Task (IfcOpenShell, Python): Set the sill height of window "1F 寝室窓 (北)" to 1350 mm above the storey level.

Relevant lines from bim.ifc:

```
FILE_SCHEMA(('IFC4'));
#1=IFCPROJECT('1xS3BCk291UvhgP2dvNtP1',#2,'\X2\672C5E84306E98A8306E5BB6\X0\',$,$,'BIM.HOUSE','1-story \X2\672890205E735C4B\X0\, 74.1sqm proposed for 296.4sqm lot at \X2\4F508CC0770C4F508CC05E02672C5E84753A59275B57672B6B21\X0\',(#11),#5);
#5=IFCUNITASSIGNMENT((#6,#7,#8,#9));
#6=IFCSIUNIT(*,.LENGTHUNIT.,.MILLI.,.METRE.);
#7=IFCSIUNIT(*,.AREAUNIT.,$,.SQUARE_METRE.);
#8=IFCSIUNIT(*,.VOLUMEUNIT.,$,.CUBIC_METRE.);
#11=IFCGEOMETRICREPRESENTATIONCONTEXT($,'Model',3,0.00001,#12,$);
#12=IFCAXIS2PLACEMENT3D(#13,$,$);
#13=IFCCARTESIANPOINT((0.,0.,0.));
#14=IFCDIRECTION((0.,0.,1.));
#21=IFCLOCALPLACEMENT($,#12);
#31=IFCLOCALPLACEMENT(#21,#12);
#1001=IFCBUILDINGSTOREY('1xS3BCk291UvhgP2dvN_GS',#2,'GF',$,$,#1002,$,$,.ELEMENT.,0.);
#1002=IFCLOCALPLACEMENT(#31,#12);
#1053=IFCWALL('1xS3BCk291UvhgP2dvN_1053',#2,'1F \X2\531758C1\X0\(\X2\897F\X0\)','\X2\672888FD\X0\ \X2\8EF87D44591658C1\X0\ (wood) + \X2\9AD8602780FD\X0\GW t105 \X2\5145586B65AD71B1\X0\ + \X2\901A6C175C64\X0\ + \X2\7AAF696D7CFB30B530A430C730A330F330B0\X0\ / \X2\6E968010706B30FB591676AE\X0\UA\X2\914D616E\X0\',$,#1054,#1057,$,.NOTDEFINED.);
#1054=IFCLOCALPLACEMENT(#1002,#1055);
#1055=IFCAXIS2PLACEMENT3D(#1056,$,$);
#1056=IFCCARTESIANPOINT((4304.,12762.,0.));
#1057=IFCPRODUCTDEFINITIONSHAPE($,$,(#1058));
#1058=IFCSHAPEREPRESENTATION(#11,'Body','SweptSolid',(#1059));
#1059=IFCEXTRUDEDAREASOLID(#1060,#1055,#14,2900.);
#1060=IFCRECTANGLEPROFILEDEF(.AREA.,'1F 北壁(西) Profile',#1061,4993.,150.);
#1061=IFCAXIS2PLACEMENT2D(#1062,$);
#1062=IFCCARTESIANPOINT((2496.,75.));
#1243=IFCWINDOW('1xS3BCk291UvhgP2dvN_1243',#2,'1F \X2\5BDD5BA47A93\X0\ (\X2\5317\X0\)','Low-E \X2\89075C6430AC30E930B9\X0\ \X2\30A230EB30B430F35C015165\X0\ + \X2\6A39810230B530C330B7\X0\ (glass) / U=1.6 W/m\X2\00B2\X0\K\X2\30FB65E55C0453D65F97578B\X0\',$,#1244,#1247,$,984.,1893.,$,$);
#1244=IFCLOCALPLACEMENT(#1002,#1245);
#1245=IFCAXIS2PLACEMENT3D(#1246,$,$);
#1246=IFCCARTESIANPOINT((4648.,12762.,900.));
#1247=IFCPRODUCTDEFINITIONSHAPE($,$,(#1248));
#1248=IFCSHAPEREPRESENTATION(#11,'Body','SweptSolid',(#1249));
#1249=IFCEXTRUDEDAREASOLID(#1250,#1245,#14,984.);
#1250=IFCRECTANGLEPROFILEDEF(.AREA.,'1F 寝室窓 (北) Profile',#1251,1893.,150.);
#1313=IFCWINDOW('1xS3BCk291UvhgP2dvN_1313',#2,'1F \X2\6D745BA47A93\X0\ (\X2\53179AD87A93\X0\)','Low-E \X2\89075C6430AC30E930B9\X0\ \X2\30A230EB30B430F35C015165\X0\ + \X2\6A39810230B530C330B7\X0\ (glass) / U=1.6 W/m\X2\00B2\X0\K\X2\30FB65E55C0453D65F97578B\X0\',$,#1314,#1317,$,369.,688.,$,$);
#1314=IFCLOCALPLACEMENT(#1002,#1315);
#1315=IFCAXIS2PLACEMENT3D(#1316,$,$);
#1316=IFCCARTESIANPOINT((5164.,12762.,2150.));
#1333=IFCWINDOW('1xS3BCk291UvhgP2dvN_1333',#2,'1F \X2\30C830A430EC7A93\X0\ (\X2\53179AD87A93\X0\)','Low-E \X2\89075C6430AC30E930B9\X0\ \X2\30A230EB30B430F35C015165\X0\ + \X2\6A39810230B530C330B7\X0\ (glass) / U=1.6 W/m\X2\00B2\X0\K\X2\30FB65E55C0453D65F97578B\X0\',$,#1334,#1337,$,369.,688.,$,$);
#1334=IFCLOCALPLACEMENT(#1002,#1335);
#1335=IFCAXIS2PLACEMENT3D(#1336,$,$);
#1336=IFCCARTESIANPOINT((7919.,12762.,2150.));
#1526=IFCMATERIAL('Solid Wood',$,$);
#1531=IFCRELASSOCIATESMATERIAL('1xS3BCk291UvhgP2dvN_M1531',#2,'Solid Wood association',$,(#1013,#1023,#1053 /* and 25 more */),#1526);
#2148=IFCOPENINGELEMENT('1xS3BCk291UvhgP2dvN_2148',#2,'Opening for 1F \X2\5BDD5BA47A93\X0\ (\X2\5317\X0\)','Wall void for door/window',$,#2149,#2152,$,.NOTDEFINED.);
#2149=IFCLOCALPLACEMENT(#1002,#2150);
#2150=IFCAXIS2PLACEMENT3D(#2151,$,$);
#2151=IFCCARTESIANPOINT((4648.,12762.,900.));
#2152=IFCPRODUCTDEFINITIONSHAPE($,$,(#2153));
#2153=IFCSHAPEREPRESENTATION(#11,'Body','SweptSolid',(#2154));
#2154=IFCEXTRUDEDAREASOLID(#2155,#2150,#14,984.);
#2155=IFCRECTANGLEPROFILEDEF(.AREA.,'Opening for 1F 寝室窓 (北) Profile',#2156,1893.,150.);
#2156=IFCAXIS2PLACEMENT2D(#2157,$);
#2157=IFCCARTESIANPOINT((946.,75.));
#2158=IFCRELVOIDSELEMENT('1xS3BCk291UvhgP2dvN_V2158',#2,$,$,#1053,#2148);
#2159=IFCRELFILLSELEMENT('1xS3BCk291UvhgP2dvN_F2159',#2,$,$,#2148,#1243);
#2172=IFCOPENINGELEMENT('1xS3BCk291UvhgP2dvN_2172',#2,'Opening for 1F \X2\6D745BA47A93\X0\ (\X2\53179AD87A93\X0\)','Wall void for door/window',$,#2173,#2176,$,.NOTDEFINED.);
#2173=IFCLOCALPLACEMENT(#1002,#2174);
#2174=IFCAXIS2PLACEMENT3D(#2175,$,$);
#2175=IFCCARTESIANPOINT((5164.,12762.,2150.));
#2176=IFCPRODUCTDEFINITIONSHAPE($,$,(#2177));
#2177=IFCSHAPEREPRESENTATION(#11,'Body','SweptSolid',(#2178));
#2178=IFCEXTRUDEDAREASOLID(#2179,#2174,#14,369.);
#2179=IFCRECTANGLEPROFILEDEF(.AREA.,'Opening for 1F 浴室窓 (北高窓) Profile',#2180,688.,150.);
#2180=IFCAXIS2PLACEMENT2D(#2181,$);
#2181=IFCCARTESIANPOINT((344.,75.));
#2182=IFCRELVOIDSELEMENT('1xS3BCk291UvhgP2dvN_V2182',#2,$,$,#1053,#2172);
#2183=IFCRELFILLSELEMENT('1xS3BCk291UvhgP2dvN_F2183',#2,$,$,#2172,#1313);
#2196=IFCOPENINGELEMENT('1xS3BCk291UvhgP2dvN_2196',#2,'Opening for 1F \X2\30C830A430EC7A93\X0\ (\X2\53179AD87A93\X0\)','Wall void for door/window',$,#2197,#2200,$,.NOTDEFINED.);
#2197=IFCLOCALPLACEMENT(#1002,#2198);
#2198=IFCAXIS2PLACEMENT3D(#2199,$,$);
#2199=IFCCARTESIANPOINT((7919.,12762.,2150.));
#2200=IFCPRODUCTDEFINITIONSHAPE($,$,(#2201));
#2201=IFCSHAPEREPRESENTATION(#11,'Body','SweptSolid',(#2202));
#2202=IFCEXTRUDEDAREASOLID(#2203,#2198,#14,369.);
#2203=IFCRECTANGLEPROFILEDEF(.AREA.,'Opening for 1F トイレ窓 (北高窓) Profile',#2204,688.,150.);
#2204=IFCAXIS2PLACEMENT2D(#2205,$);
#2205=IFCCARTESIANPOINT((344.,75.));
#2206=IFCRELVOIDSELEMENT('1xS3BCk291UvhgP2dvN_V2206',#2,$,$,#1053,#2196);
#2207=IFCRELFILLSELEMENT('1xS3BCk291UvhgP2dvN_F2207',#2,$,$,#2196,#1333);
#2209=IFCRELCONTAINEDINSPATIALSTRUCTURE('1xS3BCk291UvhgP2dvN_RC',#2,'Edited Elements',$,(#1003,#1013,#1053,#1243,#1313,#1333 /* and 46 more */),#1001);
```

```python
import numpy as np
import ifcopenshell
import ifcopenshell.api.geometry
import ifcopenshell.geom
import ifcopenshell.util.element
import ifcopenshell.util.placement
import ifcopenshell.util.shape
import ifcopenshell.util.unit

model = ifcopenshell.open("bim.ifc")
unit_scale = ifcopenshell.util.unit.calculate_unit_scale(model)

window = model.by_guid("1xS3BCk291UvhgP2dvN_1243")
opening = window.FillsVoids[0].RelatingOpeningElement
storey = ifcopenshell.util.element.get_container(window, ifc_class="IfcBuildingStorey")
level = ifcopenshell.util.placement.get_local_placement(storey.ObjectPlacement)[2, 3]

# The opening's origin need not be at the sill, so measure its lowest point.
shape = ifcopenshell.geom.create_shape(ifcopenshell.geom.settings(), opening)
bottom = ifcopenshell.util.shape.get_shape_bottom_elevation(shape, shape.geometry) / unit_scale
dz = level + 1350.0 - bottom

shift = np.array([0.0, 0.0, dz])
# The window is not placed relative to its opening, so move both.
for product in (opening, window):
    matrix = ifcopenshell.util.placement.get_local_placement(product.ObjectPlacement)
    matrix[:3, 3] += shift
    ifcopenshell.api.geometry.edit_object_placement(model, product=product, matrix=matrix, is_si=False)

print(f"moved by {dz * unit_scale:+.3f} m")

model.write("bim_v2.ifc")
```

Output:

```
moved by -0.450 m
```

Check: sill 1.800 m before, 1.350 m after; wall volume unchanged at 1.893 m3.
